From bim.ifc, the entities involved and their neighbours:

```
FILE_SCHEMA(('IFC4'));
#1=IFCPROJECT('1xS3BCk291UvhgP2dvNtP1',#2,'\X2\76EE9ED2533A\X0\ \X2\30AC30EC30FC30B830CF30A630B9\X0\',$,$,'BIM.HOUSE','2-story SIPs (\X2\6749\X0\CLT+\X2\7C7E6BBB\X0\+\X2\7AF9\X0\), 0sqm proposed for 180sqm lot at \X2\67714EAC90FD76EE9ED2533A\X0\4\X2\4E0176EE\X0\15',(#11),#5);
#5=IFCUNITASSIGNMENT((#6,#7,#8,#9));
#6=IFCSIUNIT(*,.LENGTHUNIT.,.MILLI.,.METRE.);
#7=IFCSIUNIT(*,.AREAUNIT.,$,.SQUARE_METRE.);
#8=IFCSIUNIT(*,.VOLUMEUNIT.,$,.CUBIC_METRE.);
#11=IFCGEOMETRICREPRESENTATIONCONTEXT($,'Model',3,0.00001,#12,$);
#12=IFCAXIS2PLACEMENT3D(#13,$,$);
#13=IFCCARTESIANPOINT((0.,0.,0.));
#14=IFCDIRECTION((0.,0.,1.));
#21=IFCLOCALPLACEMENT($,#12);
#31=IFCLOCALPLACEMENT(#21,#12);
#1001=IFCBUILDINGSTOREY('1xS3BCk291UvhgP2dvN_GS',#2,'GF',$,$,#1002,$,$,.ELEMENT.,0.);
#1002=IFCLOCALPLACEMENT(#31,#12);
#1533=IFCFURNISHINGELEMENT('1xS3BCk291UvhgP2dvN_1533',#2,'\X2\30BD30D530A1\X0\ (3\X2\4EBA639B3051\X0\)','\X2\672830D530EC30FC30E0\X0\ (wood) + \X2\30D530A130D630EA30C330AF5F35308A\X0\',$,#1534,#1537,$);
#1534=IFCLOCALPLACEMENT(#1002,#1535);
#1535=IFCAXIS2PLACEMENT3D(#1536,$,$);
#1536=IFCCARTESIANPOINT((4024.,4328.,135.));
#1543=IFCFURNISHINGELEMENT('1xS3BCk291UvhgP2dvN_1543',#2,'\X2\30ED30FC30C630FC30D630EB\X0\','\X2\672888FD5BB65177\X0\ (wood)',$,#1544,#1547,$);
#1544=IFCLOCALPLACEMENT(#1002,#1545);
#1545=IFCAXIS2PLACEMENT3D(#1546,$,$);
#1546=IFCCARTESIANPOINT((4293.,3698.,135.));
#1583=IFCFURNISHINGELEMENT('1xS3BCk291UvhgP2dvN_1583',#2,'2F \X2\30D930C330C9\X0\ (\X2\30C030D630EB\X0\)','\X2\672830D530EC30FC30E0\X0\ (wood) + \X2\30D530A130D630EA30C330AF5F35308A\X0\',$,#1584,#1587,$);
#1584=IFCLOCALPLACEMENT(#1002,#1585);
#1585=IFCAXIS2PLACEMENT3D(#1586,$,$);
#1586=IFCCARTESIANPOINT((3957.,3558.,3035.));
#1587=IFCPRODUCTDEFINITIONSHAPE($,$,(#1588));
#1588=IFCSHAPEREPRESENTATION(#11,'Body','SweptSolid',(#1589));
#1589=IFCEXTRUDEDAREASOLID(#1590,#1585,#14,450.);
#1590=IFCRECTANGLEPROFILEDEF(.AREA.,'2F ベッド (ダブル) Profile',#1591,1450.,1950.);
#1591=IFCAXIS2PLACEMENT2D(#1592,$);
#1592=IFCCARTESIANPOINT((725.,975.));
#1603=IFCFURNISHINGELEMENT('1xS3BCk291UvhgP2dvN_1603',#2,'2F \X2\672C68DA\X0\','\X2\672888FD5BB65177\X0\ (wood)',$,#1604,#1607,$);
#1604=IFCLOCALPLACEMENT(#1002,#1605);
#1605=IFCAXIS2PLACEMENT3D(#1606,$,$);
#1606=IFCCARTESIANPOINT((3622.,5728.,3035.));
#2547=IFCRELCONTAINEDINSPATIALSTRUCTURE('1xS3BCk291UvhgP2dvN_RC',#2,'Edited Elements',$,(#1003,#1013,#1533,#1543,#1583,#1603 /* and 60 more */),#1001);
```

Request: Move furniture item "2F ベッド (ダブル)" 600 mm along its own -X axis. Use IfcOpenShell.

```python
import ifcopenshell
import ifcopenshell.api.geometry
import ifcopenshell.util.placement

model = ifcopenshell.open("bim.ifc")

item = model.by_guid("1xS3BCk291UvhgP2dvN_1583")
matrix = ifcopenshell.util.placement.get_local_placement(item.ObjectPlacement)
matrix[:3, 3] -= matrix[:3, 0] * 600.0
ifcopenshell.api.geometry.edit_object_placement(model, product=item, matrix=matrix, is_si=False)

print(ifcopenshell.util.placement.get_local_placement(item.ObjectPlacement).round(3) + 0.0)

model.write("bim-out.ifc")
```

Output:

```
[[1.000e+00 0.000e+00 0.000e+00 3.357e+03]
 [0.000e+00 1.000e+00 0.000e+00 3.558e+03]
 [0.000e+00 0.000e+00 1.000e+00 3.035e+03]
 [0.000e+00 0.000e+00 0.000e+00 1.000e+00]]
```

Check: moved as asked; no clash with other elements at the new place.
